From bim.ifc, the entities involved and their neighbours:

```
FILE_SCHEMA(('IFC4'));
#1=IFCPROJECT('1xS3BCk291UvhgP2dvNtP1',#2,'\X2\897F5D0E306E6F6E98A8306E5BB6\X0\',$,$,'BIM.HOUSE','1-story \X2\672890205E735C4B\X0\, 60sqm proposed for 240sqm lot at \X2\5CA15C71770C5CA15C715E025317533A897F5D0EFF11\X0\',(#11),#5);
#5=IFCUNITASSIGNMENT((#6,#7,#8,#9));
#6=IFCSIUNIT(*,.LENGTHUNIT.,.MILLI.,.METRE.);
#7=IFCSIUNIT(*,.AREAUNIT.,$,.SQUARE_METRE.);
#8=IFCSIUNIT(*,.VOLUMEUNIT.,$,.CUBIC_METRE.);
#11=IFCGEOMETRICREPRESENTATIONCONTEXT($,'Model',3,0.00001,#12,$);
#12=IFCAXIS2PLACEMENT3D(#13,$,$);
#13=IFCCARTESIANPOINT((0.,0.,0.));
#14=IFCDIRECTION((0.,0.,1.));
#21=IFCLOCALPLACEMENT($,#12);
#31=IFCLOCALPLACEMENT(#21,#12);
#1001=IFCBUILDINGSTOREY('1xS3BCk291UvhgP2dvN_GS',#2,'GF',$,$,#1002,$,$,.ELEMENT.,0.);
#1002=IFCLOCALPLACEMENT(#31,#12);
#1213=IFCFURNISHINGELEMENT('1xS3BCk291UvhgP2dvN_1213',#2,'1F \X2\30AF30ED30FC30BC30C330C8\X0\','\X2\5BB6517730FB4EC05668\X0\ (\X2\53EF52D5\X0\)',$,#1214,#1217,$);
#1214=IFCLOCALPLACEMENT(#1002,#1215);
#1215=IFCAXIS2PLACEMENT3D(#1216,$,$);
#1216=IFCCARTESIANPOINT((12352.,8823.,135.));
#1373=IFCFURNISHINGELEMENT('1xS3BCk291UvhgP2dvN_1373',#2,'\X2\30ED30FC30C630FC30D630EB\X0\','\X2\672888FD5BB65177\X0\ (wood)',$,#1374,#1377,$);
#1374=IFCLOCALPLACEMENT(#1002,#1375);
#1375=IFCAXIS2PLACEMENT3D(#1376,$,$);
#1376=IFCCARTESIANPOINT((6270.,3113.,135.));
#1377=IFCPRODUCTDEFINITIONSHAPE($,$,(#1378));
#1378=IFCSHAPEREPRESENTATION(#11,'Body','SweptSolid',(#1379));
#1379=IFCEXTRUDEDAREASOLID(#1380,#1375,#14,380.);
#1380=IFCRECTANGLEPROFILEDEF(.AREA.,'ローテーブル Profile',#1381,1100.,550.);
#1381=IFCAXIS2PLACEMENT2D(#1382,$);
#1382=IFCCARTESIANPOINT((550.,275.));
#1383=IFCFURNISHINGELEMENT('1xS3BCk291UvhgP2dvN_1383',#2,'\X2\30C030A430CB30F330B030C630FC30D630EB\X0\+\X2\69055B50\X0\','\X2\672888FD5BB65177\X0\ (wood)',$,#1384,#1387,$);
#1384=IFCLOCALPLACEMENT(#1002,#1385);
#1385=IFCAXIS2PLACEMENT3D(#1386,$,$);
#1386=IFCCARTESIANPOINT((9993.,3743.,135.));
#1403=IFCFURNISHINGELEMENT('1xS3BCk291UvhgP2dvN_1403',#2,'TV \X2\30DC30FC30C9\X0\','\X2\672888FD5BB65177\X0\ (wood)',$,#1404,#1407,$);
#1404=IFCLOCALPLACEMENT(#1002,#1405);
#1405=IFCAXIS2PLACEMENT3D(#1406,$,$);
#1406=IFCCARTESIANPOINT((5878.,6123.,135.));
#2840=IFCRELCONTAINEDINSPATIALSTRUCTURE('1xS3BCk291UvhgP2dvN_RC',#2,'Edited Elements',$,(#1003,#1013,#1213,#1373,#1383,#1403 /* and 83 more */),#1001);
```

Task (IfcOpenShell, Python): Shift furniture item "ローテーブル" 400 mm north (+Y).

```python
import ifcopenshell
import ifcopenshell.api.geometry
import ifcopenshell.util.placement
import ifcopenshell.util.unit

model = ifcopenshell.open("bim.ifc")
unit_scale = ifcopenshell.util.unit.calculate_unit_scale(model)

item = model.by_guid("1xS3BCk291UvhgP2dvN_1373")
matrix = ifcopenshell.util.placement.get_local_placement(item.ObjectPlacement)
matrix[1, 3] += 0.4 / unit_scale
ifcopenshell.api.geometry.edit_object_placement(model, product=item, matrix=matrix, is_si=False)

print(ifcopenshell.util.placement.get_local_placement(item.ObjectPlacement).round(3) + 0.0)

model.write("bim_rev.ifc")
```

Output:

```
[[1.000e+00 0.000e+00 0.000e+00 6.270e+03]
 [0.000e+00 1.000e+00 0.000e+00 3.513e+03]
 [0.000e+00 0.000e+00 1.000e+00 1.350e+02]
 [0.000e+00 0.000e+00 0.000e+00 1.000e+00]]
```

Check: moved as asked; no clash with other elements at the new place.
